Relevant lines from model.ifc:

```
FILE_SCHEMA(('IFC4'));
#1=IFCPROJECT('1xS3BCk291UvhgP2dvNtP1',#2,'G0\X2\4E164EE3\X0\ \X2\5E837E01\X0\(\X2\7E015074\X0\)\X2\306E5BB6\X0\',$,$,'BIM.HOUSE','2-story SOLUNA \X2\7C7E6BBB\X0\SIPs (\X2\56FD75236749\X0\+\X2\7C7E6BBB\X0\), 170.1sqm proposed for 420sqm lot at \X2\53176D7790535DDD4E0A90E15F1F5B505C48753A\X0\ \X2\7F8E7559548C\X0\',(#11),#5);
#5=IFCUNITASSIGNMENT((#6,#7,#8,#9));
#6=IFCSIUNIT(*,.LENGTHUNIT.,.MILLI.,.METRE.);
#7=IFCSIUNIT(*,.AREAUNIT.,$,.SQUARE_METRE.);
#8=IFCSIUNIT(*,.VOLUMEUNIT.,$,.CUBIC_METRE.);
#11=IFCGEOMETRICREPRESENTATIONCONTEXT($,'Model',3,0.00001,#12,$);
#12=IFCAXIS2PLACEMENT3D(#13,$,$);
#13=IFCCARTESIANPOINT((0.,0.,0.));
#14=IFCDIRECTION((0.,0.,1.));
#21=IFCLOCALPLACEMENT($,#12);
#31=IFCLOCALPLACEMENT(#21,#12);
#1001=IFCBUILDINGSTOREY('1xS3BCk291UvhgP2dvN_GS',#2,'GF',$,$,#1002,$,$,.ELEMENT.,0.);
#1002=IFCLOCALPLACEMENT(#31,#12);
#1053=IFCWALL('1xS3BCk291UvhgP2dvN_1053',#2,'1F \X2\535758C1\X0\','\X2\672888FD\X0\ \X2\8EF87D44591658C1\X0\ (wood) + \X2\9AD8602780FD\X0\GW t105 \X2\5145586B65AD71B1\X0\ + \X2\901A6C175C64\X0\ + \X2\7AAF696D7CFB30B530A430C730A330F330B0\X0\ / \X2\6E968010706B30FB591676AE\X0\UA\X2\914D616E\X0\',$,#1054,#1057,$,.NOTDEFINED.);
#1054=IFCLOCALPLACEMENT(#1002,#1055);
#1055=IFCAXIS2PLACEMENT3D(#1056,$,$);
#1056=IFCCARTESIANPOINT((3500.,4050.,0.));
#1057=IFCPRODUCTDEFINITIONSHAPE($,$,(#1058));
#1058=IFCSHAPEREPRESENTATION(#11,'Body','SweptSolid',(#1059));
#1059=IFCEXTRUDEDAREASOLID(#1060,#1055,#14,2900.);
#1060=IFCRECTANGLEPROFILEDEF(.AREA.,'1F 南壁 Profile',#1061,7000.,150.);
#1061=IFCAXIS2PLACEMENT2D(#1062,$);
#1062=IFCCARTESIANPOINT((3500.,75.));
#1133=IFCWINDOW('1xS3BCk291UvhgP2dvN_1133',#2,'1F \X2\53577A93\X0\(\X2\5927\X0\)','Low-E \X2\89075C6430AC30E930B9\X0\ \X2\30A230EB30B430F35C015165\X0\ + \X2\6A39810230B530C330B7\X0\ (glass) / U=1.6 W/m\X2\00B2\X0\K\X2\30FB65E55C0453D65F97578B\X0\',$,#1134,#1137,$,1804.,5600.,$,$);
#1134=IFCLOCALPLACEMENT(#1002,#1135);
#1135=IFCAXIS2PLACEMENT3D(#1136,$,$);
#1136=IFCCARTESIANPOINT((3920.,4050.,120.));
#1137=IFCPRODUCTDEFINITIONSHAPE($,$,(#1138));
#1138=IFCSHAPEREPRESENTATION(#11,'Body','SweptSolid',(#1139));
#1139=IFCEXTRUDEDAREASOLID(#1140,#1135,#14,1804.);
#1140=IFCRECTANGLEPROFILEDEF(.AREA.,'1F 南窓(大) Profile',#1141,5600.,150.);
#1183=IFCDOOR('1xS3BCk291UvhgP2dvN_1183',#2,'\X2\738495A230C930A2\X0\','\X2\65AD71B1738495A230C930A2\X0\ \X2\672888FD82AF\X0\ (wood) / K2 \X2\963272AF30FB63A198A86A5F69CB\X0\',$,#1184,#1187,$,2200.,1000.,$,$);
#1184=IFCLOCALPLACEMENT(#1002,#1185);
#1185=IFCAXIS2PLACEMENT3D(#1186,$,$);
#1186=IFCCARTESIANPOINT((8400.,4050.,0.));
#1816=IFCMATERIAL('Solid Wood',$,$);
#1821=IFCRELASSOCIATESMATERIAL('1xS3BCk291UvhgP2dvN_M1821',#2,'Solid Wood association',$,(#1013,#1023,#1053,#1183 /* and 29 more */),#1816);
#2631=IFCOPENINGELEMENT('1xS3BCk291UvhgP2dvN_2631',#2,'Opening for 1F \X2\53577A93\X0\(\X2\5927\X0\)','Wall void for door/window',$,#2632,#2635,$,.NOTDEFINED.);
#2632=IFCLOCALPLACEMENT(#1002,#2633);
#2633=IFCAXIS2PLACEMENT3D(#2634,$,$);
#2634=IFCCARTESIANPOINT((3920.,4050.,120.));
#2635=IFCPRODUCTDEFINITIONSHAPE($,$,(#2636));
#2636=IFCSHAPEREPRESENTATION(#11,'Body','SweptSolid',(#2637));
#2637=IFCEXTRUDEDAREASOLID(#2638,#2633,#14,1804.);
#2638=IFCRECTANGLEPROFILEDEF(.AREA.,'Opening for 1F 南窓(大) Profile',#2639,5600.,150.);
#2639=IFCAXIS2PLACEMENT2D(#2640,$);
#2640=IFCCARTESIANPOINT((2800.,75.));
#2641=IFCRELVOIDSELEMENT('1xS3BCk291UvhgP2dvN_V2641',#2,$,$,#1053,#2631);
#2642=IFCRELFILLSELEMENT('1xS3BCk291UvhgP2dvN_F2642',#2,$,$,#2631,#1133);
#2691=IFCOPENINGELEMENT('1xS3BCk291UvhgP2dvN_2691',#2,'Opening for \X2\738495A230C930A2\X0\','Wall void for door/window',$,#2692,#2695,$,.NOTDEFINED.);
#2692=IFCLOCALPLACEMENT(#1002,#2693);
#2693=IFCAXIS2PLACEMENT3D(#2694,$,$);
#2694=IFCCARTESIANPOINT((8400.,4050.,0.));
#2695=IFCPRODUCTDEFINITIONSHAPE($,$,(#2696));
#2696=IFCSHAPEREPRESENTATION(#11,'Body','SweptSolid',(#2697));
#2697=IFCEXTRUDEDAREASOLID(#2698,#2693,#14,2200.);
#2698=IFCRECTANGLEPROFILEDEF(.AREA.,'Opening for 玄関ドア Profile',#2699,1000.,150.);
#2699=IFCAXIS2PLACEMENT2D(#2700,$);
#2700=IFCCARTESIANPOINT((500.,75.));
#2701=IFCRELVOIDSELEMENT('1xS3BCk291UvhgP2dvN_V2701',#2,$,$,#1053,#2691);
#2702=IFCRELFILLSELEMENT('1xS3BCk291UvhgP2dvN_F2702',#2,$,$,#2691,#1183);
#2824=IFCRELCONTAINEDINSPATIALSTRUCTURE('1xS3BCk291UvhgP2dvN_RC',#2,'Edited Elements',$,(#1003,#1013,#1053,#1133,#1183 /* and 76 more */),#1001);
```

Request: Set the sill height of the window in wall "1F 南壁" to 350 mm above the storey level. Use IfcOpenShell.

```python
import numpy as np
import ifcopenshell
import ifcopenshell.api.geometry
import ifcopenshell.geom
import ifcopenshell.util.element
import ifcopenshell.util.placement
import ifcopenshell.util.shape
import ifcopenshell.util.unit

model = ifcopenshell.open("model.ifc")
unit_scale = ifcopenshell.util.unit.calculate_unit_scale(model)

window = model.by_guid("1xS3BCk291UvhgP2dvN_1133")
opening = window.FillsVoids[0].RelatingOpeningElement
storey = ifcopenshell.util.element.get_container(window, ifc_class="IfcBuildingStorey")
level = ifcopenshell.util.placement.get_local_placement(storey.ObjectPlacement)[2, 3]

# The opening's origin need not be at the sill, so measure its lowest point.
shape = ifcopenshell.geom.create_shape(ifcopenshell.geom.settings(), opening)
bottom = ifcopenshell.util.shape.get_shape_bottom_elevation(shape, shape.geometry) / unit_scale
dz = level + 350.0 - bottom

shift = np.array([0.0, 0.0, dz])
# The window is not placed relative to its opening, so move both.
for product in (opening, window):
    matrix = ifcopenshell.util.placement.get_local_placement(product.ObjectPlacement)
    matrix[:3, 3] += shift
    ifcopenshell.api.geometry.edit_object_placement(model, product=product, matrix=matrix, is_si=False)

print(f"moved by {dz * unit_scale:+.3f} m")

model.write("model_rev.ifc")
```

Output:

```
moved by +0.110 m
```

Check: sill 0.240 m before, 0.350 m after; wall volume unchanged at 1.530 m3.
